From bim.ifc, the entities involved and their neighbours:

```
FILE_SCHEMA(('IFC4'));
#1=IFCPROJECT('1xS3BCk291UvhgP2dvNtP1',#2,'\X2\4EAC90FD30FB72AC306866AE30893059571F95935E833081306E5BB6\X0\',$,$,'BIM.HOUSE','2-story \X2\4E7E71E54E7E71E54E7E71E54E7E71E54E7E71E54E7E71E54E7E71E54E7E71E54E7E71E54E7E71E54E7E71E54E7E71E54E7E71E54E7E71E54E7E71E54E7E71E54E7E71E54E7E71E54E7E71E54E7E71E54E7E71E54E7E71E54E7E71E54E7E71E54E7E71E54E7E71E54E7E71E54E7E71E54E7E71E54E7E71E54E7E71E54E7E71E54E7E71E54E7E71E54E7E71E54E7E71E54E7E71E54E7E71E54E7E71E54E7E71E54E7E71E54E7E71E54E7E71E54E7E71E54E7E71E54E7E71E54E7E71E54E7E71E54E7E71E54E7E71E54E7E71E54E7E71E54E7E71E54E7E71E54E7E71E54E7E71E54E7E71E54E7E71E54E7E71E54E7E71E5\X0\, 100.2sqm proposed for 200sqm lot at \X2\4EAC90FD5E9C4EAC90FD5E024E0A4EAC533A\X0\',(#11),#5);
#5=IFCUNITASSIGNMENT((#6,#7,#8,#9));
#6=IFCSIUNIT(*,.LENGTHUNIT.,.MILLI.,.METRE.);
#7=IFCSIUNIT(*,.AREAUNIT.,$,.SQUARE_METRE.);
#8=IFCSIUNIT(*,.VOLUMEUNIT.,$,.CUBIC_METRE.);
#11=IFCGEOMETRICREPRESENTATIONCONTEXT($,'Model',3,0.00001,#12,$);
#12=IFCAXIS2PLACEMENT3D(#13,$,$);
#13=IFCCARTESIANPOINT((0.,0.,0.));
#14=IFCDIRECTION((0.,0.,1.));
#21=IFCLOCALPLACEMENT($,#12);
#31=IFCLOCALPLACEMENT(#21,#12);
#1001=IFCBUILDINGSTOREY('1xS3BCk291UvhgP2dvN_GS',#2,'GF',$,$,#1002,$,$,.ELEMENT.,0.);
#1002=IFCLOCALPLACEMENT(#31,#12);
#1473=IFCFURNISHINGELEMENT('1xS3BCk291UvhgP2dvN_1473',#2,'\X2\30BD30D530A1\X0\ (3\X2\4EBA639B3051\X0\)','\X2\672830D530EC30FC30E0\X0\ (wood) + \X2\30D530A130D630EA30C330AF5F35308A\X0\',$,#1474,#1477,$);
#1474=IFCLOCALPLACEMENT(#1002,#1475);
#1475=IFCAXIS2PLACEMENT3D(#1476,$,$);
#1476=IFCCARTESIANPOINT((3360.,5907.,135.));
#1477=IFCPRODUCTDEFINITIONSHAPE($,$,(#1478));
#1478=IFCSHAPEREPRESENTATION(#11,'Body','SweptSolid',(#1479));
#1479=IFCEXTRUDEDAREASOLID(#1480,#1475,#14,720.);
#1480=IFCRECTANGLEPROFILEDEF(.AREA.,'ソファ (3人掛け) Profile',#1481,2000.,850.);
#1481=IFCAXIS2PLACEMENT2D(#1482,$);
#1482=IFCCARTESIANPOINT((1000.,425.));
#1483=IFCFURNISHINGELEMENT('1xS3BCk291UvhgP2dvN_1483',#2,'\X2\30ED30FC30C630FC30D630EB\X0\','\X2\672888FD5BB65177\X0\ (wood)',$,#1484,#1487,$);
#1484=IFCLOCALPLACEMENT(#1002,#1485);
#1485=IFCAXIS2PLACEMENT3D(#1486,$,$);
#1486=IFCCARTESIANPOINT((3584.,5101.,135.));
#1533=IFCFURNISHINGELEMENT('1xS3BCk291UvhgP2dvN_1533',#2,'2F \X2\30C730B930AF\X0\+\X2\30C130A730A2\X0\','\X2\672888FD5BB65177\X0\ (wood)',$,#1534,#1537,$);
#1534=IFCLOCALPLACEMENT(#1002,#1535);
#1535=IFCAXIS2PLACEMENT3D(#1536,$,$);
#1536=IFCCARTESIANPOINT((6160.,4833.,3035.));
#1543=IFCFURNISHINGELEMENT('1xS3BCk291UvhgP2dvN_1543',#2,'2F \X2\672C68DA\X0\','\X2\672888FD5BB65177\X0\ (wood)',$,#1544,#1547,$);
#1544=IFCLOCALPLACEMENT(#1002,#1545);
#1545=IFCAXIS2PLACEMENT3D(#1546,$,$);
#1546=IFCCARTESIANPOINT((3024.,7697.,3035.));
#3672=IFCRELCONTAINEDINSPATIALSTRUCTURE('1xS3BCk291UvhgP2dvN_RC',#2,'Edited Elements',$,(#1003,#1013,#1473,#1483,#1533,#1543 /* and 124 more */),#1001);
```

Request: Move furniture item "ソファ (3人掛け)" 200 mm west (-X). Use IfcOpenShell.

```python
import ifcopenshell
import ifcopenshell.api.geometry
import ifcopenshell.util.placement

model = ifcopenshell.open("bim.ifc")

item = model.by_guid("1xS3BCk291UvhgP2dvN_1473")
matrix = ifcopenshell.util.placement.get_local_placement(item.ObjectPlacement)
matrix[0, 3] -= 200.0
ifcopenshell.api.geometry.edit_object_placement(model, product=item, matrix=matrix, is_si=False)

print(ifcopenshell.util.placement.get_local_placement(item.ObjectPlacement).round(3) + 0.0)

model.write("bim-out.ifc")
```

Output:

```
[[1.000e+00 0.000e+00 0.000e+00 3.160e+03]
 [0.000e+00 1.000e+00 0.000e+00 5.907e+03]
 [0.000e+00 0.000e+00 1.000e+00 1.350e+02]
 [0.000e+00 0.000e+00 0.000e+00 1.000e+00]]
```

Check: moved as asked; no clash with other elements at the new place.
